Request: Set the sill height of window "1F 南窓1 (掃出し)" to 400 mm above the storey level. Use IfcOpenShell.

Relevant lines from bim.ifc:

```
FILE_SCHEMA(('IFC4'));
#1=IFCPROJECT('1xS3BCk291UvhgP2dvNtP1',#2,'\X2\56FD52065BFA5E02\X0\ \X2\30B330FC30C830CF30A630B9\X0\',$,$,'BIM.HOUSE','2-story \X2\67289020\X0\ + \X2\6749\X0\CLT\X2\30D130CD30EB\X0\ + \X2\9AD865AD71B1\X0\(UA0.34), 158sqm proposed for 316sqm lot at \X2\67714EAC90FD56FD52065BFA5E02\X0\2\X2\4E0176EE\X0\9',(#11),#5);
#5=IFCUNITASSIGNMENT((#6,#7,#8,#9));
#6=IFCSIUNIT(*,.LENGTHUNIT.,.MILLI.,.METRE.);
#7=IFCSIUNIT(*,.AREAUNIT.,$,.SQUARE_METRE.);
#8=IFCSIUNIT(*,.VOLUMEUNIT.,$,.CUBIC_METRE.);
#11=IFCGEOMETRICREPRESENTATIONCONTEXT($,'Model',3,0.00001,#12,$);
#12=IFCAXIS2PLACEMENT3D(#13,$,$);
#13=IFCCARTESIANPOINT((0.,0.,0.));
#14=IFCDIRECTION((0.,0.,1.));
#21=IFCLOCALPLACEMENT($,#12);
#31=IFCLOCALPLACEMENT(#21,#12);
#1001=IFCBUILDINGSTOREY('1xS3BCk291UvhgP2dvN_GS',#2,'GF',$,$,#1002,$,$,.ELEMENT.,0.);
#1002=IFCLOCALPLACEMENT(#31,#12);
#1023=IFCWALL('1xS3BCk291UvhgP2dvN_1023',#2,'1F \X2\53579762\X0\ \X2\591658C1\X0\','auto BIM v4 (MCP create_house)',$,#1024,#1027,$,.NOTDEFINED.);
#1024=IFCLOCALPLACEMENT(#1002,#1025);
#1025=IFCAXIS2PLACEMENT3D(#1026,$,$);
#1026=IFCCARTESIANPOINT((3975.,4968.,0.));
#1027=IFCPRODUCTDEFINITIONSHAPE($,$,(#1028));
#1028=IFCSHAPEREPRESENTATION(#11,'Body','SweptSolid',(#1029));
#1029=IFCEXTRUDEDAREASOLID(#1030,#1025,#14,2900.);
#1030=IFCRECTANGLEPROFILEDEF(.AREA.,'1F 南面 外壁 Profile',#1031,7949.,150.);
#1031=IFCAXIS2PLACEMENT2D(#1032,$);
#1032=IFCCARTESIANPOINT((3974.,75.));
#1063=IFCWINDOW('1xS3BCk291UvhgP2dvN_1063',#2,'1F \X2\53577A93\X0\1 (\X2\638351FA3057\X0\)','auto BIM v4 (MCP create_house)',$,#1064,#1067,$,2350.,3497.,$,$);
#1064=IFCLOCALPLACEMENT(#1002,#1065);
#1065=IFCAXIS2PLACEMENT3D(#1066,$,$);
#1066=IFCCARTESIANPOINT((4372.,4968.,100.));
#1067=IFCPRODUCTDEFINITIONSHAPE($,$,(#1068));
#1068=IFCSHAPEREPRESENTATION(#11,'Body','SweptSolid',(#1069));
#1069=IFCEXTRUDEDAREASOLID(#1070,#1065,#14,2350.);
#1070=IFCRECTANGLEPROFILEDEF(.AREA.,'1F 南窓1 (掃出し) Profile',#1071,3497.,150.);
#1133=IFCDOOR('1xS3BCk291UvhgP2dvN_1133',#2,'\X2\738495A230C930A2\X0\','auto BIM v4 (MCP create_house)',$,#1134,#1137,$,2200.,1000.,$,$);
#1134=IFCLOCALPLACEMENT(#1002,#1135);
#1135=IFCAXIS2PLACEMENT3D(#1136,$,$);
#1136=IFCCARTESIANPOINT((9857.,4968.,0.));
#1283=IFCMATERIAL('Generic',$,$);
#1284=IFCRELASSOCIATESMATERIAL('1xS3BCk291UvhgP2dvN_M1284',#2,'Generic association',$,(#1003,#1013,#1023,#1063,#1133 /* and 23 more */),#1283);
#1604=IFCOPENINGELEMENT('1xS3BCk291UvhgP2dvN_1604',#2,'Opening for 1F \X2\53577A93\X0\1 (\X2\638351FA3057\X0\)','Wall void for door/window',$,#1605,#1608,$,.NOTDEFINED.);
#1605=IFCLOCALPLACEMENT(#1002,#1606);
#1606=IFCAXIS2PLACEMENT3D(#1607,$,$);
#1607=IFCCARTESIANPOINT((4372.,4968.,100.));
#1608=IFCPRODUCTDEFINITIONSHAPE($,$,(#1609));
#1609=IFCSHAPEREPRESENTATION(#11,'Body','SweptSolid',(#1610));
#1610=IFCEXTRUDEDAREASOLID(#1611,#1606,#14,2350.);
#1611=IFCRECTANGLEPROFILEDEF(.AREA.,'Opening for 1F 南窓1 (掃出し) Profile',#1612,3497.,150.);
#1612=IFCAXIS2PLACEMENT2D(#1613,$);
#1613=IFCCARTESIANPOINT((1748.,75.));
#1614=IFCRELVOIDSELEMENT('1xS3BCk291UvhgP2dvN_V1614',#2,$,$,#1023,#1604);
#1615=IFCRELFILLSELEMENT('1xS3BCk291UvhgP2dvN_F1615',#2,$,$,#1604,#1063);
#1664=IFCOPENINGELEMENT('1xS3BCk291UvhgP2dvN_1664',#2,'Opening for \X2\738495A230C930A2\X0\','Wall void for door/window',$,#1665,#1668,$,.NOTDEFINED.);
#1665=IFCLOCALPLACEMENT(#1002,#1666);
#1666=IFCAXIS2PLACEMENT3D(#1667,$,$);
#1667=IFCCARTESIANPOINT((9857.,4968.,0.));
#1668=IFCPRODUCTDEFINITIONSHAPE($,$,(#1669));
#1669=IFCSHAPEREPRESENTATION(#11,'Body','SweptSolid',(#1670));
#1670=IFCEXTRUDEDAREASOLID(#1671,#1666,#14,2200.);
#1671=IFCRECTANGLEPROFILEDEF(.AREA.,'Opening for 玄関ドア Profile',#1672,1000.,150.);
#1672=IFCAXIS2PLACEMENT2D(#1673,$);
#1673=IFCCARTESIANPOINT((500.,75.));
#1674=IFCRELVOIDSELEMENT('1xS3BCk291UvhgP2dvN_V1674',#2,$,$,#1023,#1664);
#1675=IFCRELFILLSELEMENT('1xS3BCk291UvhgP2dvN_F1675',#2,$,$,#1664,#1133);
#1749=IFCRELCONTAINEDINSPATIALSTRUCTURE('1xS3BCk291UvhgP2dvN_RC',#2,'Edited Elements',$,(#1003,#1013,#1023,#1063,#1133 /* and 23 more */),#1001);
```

```python
import numpy as np
import ifcopenshell
import ifcopenshell.api.geometry
import ifcopenshell.geom
import ifcopenshell.util.element
import ifcopenshell.util.placement
import ifcopenshell.util.shape
import ifcopenshell.util.unit

model = ifcopenshell.open("bim.ifc")
unit_scale = ifcopenshell.util.unit.calculate_unit_scale(model)

window = model.by_guid("1xS3BCk291UvhgP2dvN_1063")
opening = window.FillsVoids[0].RelatingOpeningElement
storey = ifcopenshell.util.element.get_container(window, ifc_class="IfcBuildingStorey")
level = ifcopenshell.util.placement.get_local_placement(storey.ObjectPlacement)[2, 3]

# The opening's origin need not be at the sill, so measure its lowest point.
shape = ifcopenshell.geom.create_shape(ifcopenshell.geom.settings(), opening)
bottom = ifcopenshell.util.shape.get_shape_bottom_elevation(shape, shape.geometry) / unit_scale
dz = level + 400.0 - bottom

shift = np.array([0.0, 0.0, dz])
# The window is not placed relative to its opening, so move both.
for product in (opening, window):
    matrix = ifcopenshell.util.placement.get_local_placement(product.ObjectPlacement)
    matrix[:3, 3] += shift
    ifcopenshell.api.geometry.edit_object_placement(model, product=product, matrix=matrix, is_si=False)

print(f"moved by {dz * unit_scale:+.3f} m")

model.write("bim_edited.ifc")
```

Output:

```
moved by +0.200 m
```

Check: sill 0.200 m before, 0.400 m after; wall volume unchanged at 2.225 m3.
